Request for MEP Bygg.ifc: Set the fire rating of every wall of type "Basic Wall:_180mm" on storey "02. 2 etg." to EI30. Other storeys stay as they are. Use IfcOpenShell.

First a look at what the model holds.

```python
import ifcopenshell
import ifcopenshell.util.element

model = ifcopenshell.open("MEP Bygg.ifc")
print(model.schema)
storey = next(s for s in model.by_type("IfcBuildingStorey") if s.Name == "02. 2 etg.")
walls = [e for e in ifcopenshell.util.element.get_decomposition(storey) if e.is_a("IfcWall")]
seen = {}
for e in walls:
    element_type = ifcopenshell.util.element.get_type(e)
    key = (element_type.Name if element_type != e and element_type else None, ifcopenshell.util.element.get_pset(e, "Pset_WallCommon", "FireRating"))
    seen[key] = seen.get(key, 0) + 1
for (name, value), count in sorted(seen.items(), key=str):
    print(count, "x", name, "|", value)
```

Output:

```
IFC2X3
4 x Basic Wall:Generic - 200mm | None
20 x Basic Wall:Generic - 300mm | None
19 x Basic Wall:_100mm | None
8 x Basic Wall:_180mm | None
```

```python
import ifcopenshell
import ifcopenshell.api.pset
import ifcopenshell.util.element

model = ifcopenshell.open("MEP Bygg.ifc")

storey = next(s for s in model.by_type("IfcBuildingStorey") if s.Name == "02. 2 etg.")
walls = [e for e in ifcopenshell.util.element.get_decomposition(storey) if e.is_a("IfcWall")]

count = 0
for e in walls:
    element_type = ifcopenshell.util.element.get_type(e)
    if element_type in (None, e) or element_type.Name != "Basic Wall:_180mm":
        continue
    # add_pset returns the element's existing set when there is one.
    pset = ifcopenshell.api.pset.add_pset(model, product=e, name="Pset_WallCommon")
    ifcopenshell.api.pset.edit_pset(model, pset=pset, properties={"FireRating": "EI30"})
    count += 1

print(count, "walls updated")

model.write("MEP Bygg-out.ifc")
```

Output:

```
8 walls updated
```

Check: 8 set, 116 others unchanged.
